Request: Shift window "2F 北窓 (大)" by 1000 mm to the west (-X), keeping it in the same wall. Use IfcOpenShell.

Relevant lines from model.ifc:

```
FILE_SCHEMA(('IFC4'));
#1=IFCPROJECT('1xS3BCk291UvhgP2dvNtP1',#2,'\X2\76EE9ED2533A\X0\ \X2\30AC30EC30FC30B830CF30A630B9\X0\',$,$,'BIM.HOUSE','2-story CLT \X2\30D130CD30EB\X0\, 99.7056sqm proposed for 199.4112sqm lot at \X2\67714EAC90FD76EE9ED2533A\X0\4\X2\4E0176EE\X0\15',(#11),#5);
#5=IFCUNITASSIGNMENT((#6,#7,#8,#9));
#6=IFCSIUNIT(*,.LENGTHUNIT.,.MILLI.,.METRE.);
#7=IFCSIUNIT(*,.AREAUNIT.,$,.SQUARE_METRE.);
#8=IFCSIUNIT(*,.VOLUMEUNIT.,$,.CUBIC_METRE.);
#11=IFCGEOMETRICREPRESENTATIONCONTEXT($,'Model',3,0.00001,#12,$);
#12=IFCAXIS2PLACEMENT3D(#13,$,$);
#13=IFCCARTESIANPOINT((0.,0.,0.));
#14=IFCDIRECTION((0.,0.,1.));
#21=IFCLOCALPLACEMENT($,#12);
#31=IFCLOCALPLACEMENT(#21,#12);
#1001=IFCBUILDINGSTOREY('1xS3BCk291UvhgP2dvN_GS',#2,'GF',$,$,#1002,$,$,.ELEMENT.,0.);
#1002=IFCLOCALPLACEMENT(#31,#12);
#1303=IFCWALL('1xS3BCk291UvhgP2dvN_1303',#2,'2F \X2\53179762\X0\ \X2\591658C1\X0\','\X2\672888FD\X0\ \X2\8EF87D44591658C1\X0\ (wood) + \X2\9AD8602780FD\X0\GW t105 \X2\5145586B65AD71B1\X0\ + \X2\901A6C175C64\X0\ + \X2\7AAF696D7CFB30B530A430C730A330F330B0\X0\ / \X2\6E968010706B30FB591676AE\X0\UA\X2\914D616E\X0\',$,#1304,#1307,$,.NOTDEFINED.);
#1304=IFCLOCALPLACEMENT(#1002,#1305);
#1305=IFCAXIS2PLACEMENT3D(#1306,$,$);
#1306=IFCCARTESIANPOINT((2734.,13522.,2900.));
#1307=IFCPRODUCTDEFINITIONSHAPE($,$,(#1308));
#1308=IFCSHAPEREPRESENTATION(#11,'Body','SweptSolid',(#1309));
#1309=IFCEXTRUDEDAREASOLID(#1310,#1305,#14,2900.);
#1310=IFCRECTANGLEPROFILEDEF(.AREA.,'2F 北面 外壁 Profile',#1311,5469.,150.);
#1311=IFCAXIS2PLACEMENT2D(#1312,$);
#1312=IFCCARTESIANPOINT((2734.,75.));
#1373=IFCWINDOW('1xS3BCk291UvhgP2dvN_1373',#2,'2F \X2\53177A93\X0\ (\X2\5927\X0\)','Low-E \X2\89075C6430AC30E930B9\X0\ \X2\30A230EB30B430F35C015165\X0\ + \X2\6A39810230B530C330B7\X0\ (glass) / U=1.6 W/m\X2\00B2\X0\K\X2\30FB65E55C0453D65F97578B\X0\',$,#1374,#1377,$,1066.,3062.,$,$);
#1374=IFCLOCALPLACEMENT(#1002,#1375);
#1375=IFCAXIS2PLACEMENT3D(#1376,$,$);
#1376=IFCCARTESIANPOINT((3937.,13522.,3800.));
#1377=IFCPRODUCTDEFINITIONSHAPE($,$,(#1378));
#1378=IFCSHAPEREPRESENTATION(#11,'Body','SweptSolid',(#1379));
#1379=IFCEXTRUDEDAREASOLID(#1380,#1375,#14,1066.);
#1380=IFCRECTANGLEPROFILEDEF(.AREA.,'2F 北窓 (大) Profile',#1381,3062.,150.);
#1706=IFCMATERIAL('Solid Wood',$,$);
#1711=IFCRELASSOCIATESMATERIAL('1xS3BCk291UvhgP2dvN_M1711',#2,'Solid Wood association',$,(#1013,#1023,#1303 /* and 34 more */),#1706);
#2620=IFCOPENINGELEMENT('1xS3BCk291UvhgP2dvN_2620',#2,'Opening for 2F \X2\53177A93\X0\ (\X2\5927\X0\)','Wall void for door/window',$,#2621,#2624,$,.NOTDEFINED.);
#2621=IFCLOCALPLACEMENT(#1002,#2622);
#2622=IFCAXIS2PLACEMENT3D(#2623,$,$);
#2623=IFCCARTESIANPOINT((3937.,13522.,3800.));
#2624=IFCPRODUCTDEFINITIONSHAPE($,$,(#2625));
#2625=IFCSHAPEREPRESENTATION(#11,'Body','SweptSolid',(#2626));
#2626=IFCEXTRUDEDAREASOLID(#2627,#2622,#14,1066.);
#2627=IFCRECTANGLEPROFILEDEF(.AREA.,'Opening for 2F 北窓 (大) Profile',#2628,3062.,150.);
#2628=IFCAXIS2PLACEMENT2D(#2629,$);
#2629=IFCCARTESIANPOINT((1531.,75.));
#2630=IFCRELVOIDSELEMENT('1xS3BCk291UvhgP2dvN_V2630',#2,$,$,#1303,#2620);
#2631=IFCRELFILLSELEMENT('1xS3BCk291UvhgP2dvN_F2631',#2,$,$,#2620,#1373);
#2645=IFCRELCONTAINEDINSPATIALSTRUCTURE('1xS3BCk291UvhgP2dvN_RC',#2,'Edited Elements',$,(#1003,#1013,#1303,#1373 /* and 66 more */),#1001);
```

```python
import ifcopenshell
import ifcopenshell.api.geometry
import ifcopenshell.util.placement
import ifcopenshell.util.unit

model = ifcopenshell.open("model.ifc")
unit_scale = ifcopenshell.util.unit.calculate_unit_scale(model)

window = model.by_id(1373)
opening = window.FillsVoids[0].RelatingOpeningElement
wall = opening.VoidsElements[0].RelatingBuildingElement

wall_matrix = ifcopenshell.util.placement.get_local_placement(wall.ObjectPlacement)
shift = wall_matrix[:3, 0] * -1 / unit_scale
before = ifcopenshell.util.placement.get_local_placement(window.ObjectPlacement)[:3, 3].copy()

# The window is not placed relative to its opening, so move both.
for product in (opening, window):
    matrix = ifcopenshell.util.placement.get_local_placement(product.ObjectPlacement)
    matrix[:3, 3] += shift
    ifcopenshell.api.geometry.edit_object_placement(model, product=product, matrix=matrix, is_si=False)

after = ifcopenshell.util.placement.get_local_placement(window.ObjectPlacement)[:3, 3]
print("window moved by", (after - before).round(3) + 0.0)

model.write("model_updated.ifc")
```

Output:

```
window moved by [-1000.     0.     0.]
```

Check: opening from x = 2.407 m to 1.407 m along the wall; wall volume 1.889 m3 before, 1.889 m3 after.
